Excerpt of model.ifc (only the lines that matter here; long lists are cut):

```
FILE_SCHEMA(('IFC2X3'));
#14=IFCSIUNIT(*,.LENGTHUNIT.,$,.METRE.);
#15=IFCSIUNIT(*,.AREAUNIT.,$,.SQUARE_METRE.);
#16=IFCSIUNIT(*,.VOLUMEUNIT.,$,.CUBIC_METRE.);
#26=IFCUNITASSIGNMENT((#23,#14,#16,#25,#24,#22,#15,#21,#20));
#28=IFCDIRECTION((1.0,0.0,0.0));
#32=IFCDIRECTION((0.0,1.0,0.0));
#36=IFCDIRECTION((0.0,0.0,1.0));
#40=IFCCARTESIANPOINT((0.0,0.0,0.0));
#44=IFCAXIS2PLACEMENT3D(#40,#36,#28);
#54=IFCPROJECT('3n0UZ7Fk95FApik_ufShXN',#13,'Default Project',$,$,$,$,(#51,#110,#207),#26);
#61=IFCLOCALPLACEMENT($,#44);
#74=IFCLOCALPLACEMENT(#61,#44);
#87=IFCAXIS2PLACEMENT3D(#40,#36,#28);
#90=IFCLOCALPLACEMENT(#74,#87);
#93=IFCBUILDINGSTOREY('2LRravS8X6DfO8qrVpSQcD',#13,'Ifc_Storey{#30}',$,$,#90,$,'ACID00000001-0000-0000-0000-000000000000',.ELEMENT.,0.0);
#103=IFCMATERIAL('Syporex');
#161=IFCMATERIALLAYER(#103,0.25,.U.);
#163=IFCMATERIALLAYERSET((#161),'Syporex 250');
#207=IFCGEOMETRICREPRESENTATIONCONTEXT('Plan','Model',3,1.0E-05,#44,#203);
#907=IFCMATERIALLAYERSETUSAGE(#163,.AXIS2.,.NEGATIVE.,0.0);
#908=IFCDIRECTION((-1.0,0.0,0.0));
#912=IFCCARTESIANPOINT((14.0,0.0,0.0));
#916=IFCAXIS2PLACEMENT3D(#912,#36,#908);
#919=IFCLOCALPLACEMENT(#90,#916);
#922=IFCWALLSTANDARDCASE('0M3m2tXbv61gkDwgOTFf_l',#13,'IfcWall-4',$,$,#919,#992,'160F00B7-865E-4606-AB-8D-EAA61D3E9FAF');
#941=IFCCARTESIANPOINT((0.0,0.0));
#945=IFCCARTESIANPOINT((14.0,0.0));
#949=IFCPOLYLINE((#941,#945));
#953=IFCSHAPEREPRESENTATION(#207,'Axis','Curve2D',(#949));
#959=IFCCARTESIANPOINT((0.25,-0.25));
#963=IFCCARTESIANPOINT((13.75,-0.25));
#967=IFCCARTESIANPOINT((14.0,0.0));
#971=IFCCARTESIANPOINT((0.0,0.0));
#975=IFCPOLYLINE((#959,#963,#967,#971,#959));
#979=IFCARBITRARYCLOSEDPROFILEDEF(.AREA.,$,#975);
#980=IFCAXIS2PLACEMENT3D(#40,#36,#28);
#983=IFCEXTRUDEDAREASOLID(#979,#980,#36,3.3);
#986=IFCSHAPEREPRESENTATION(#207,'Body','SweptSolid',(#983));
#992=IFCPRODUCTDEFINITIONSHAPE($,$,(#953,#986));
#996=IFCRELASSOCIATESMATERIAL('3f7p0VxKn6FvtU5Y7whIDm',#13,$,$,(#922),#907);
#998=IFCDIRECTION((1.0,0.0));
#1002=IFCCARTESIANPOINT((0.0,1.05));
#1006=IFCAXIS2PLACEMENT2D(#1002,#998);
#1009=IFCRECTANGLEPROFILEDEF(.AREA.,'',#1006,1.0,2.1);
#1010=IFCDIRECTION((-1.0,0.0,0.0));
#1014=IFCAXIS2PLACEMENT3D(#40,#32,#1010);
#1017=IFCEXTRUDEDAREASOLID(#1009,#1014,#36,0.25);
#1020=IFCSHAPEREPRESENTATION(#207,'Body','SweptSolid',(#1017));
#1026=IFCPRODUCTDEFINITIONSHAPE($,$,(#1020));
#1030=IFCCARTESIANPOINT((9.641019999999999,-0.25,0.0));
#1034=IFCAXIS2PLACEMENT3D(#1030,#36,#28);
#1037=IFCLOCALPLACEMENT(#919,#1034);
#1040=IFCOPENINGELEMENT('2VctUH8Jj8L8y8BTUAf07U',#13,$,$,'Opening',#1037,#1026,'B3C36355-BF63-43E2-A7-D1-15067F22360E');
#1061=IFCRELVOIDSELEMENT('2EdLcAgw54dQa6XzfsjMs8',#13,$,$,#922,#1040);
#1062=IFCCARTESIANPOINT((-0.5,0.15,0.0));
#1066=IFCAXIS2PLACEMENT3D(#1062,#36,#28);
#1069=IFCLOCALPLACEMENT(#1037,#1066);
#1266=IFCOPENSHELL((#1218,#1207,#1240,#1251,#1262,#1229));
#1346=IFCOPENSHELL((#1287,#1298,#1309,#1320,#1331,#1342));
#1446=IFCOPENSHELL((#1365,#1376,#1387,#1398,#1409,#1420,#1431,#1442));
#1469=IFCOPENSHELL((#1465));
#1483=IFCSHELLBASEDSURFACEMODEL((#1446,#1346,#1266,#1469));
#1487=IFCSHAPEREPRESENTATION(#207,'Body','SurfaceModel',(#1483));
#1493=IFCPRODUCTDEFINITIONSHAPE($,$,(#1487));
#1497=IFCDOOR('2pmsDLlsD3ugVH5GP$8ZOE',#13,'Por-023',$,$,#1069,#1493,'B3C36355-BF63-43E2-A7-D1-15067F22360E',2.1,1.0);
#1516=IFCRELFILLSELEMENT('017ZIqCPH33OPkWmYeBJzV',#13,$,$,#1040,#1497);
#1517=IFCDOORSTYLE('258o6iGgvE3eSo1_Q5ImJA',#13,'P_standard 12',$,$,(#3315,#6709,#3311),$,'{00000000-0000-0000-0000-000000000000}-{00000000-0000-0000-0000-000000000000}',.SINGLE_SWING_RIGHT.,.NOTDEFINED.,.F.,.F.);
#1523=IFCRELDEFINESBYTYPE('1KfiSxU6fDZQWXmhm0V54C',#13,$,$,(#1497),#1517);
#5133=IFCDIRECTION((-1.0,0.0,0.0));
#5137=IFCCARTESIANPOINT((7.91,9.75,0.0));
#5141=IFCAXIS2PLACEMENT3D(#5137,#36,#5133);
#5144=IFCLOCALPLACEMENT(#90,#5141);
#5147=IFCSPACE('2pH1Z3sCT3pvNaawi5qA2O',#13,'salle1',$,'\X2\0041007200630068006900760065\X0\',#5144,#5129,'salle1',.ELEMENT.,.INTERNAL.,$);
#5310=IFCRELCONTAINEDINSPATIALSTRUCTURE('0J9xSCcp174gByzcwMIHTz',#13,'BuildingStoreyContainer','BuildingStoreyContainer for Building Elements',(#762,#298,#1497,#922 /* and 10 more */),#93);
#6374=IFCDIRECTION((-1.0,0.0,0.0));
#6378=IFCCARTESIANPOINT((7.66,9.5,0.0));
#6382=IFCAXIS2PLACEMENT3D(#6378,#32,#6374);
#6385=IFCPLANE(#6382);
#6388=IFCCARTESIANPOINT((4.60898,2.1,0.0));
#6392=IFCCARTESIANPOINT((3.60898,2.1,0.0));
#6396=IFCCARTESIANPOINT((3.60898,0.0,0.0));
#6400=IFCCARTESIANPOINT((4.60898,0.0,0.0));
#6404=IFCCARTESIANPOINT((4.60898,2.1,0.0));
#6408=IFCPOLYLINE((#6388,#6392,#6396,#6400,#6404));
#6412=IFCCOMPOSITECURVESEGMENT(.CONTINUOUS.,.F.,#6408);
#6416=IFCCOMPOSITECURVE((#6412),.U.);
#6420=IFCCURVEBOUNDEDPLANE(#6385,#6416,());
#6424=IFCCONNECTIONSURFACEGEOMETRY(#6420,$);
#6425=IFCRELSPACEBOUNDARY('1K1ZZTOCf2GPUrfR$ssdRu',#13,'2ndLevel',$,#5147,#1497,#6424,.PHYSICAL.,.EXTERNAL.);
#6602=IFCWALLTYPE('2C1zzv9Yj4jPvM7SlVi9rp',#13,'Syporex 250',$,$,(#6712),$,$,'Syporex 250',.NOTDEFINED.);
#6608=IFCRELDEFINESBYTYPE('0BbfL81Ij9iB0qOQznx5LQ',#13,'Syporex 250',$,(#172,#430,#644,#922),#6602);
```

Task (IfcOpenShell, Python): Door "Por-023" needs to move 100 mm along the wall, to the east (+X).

```python
import numpy as np
import ifcopenshell
import ifcopenshell.api.geometry
import ifcopenshell.util.placement

model = ifcopenshell.open("model.ifc")

door = model.by_guid("2pmsDLlsD3ugVH5GP$8ZOE")
opening = door.FillsVoids[0].RelatingOpeningElement
wall = opening.VoidsElements[0].RelatingBuildingElement

wall_matrix = ifcopenshell.util.placement.get_local_placement(wall.ObjectPlacement)
shift = wall_matrix[:3, 0] * -0.1
before = ifcopenshell.util.placement.get_local_placement(door.ObjectPlacement)[:3, 3].copy()

# The door is placed relative to its opening, so it follows when the opening moves.
matrix = ifcopenshell.util.placement.get_local_placement(opening.ObjectPlacement)
matrix[:3, 3] += shift
ifcopenshell.api.geometry.edit_object_placement(
    model, product=opening, matrix=matrix, is_si=False, should_transform_children=True
)

# Space boundary surfaces are stored in each space's coordinates; move them too.
for rel in door.ProvidesBoundaries:
    if not rel.ConnectionGeometry:
        continue
    surface = rel.ConnectionGeometry.SurfaceOnRelatingElement.BasisSurface
    space_matrix = ifcopenshell.util.placement.get_local_placement(rel.RelatingSpace.ObjectPlacement)
    point = np.array(surface.Position.Location.Coordinates) + space_matrix[:3, :3].T @ shift
    surface.Position = model.createIfcAxis2Placement3D(
        model.createIfcCartesianPoint(point.tolist()), surface.Position.Axis, surface.Position.RefDirection
    )

after = ifcopenshell.util.placement.get_local_placement(door.ObjectPlacement)[:3, 3]
print("door moved by", (after - before).round(3) + 0.0)

model.write("model_edited.ifc")
```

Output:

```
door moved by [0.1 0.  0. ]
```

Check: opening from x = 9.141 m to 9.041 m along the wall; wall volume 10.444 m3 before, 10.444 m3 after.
